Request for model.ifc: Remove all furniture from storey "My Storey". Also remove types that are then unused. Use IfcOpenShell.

First a look at what the model holds.

```python
import ifcopenshell
import ifcopenshell.util.element

model = ifcopenshell.open("model.ifc")
print(model.schema)
storey = next(s for s in model.by_type("IfcBuildingStorey") if s.Name == "My Storey")
furniture = [e for e in ifcopenshell.util.element.get_decomposition(storey) if e.is_a("IfcFurnishingElement")]
seen = {}
for e in furniture:
    element_type = ifcopenshell.util.element.get_type(e)
    name = element_type.Name if element_type not in (None, e) else None
    seen[name] = seen.get(name, 0) + 1
for name, count in sorted(seen.items(), key=str):
    print(count, "x", name)
```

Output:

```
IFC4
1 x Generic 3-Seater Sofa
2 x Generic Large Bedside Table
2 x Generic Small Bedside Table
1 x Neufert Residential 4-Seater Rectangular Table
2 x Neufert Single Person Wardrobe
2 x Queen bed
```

```python
import ifcopenshell
import ifcopenshell.api.root
import ifcopenshell.util.element

model = ifcopenshell.open("model.ifc")

storey = next(s for s in model.by_type("IfcBuildingStorey") if s.Name == "My Storey")
furniture = [e for e in ifcopenshell.util.element.get_decomposition(storey) if e.is_a("IfcFurnishingElement")]
types = {ifcopenshell.util.element.get_type(e) for e in furniture} - {None, *furniture}

for e in furniture:
    ifcopenshell.api.root.remove_product(model, product=e)
print(len(furniture), "removed")

unused = [t for t in types if not ifcopenshell.util.element.get_types(t)]
for t in unused:
    ifcopenshell.api.root.remove_product(model, product=t)
print(len(unused), "unused types removed")

model.write("model_rev.ifc")
```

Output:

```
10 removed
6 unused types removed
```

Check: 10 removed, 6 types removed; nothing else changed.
